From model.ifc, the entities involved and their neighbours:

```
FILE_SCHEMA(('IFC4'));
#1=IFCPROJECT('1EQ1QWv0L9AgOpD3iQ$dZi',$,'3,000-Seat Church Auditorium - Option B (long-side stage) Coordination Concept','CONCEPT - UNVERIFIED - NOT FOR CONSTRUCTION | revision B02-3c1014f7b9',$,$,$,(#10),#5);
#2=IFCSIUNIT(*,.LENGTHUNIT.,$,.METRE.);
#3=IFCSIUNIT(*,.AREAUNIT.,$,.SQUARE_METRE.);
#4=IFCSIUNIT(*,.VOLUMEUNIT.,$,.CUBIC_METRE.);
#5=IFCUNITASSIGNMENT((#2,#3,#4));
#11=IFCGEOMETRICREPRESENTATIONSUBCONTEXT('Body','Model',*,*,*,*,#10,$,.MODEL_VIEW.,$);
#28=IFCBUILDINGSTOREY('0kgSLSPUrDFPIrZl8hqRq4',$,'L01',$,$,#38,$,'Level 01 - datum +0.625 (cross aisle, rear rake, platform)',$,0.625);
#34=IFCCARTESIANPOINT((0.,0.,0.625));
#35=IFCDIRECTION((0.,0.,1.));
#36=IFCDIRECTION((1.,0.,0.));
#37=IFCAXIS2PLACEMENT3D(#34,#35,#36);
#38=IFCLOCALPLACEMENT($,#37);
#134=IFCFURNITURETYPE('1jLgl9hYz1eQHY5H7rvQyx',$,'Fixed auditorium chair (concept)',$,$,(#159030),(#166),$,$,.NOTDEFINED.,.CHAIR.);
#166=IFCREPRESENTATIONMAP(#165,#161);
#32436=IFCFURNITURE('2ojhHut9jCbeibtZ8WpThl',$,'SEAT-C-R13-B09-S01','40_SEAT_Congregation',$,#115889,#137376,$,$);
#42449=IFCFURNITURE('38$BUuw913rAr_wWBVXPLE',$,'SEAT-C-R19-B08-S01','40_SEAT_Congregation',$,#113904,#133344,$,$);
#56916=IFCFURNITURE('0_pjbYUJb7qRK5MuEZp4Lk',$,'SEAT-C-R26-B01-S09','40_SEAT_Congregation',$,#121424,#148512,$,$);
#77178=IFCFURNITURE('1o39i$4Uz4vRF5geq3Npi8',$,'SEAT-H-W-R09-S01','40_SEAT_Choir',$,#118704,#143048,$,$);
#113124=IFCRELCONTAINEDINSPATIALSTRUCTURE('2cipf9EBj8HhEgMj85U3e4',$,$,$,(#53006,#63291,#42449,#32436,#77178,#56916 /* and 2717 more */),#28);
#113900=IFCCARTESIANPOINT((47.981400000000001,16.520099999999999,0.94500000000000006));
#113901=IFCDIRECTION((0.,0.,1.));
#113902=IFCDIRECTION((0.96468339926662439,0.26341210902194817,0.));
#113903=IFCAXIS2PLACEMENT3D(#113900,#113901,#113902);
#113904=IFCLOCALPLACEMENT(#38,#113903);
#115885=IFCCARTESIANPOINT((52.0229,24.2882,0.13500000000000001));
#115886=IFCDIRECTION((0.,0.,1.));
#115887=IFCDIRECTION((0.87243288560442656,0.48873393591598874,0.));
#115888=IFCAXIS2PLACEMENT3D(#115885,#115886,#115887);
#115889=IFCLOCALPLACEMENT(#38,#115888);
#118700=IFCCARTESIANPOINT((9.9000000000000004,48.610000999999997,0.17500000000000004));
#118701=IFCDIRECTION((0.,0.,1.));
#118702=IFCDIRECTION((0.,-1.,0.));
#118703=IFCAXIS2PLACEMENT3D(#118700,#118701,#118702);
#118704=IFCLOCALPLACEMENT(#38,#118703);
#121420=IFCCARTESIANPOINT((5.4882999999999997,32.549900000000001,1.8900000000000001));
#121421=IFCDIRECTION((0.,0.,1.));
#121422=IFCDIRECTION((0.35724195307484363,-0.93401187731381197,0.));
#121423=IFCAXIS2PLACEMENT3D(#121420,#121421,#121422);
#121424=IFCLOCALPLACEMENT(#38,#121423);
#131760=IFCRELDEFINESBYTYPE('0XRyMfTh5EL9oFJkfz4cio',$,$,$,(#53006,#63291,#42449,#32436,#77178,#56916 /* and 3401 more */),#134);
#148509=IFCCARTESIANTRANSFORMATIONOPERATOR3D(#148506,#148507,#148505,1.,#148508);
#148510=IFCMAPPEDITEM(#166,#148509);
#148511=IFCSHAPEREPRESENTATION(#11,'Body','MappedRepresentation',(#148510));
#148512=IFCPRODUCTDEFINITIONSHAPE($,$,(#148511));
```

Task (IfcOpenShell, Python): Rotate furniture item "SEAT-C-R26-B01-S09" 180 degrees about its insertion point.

```python
import ifcopenshell
import ifcopenshell.api.geometry
import ifcopenshell.util.placement

model = ifcopenshell.open("model.ifc")

item = model.by_guid("0_pjbYUJb7qRK5MuEZp4Lk")
matrix = ifcopenshell.util.placement.get_local_placement(item.ObjectPlacement)
matrix = matrix @ ifcopenshell.util.placement.rotation(180, "Z")
ifcopenshell.api.geometry.edit_object_placement(model, product=item, matrix=matrix, is_si=False)

print(ifcopenshell.util.placement.get_local_placement(item.ObjectPlacement).round(3) + 0.0)

model.write("model_edited.ifc")
```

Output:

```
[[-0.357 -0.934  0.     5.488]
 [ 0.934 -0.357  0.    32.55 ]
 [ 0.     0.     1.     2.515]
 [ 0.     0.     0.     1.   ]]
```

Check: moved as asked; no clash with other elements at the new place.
